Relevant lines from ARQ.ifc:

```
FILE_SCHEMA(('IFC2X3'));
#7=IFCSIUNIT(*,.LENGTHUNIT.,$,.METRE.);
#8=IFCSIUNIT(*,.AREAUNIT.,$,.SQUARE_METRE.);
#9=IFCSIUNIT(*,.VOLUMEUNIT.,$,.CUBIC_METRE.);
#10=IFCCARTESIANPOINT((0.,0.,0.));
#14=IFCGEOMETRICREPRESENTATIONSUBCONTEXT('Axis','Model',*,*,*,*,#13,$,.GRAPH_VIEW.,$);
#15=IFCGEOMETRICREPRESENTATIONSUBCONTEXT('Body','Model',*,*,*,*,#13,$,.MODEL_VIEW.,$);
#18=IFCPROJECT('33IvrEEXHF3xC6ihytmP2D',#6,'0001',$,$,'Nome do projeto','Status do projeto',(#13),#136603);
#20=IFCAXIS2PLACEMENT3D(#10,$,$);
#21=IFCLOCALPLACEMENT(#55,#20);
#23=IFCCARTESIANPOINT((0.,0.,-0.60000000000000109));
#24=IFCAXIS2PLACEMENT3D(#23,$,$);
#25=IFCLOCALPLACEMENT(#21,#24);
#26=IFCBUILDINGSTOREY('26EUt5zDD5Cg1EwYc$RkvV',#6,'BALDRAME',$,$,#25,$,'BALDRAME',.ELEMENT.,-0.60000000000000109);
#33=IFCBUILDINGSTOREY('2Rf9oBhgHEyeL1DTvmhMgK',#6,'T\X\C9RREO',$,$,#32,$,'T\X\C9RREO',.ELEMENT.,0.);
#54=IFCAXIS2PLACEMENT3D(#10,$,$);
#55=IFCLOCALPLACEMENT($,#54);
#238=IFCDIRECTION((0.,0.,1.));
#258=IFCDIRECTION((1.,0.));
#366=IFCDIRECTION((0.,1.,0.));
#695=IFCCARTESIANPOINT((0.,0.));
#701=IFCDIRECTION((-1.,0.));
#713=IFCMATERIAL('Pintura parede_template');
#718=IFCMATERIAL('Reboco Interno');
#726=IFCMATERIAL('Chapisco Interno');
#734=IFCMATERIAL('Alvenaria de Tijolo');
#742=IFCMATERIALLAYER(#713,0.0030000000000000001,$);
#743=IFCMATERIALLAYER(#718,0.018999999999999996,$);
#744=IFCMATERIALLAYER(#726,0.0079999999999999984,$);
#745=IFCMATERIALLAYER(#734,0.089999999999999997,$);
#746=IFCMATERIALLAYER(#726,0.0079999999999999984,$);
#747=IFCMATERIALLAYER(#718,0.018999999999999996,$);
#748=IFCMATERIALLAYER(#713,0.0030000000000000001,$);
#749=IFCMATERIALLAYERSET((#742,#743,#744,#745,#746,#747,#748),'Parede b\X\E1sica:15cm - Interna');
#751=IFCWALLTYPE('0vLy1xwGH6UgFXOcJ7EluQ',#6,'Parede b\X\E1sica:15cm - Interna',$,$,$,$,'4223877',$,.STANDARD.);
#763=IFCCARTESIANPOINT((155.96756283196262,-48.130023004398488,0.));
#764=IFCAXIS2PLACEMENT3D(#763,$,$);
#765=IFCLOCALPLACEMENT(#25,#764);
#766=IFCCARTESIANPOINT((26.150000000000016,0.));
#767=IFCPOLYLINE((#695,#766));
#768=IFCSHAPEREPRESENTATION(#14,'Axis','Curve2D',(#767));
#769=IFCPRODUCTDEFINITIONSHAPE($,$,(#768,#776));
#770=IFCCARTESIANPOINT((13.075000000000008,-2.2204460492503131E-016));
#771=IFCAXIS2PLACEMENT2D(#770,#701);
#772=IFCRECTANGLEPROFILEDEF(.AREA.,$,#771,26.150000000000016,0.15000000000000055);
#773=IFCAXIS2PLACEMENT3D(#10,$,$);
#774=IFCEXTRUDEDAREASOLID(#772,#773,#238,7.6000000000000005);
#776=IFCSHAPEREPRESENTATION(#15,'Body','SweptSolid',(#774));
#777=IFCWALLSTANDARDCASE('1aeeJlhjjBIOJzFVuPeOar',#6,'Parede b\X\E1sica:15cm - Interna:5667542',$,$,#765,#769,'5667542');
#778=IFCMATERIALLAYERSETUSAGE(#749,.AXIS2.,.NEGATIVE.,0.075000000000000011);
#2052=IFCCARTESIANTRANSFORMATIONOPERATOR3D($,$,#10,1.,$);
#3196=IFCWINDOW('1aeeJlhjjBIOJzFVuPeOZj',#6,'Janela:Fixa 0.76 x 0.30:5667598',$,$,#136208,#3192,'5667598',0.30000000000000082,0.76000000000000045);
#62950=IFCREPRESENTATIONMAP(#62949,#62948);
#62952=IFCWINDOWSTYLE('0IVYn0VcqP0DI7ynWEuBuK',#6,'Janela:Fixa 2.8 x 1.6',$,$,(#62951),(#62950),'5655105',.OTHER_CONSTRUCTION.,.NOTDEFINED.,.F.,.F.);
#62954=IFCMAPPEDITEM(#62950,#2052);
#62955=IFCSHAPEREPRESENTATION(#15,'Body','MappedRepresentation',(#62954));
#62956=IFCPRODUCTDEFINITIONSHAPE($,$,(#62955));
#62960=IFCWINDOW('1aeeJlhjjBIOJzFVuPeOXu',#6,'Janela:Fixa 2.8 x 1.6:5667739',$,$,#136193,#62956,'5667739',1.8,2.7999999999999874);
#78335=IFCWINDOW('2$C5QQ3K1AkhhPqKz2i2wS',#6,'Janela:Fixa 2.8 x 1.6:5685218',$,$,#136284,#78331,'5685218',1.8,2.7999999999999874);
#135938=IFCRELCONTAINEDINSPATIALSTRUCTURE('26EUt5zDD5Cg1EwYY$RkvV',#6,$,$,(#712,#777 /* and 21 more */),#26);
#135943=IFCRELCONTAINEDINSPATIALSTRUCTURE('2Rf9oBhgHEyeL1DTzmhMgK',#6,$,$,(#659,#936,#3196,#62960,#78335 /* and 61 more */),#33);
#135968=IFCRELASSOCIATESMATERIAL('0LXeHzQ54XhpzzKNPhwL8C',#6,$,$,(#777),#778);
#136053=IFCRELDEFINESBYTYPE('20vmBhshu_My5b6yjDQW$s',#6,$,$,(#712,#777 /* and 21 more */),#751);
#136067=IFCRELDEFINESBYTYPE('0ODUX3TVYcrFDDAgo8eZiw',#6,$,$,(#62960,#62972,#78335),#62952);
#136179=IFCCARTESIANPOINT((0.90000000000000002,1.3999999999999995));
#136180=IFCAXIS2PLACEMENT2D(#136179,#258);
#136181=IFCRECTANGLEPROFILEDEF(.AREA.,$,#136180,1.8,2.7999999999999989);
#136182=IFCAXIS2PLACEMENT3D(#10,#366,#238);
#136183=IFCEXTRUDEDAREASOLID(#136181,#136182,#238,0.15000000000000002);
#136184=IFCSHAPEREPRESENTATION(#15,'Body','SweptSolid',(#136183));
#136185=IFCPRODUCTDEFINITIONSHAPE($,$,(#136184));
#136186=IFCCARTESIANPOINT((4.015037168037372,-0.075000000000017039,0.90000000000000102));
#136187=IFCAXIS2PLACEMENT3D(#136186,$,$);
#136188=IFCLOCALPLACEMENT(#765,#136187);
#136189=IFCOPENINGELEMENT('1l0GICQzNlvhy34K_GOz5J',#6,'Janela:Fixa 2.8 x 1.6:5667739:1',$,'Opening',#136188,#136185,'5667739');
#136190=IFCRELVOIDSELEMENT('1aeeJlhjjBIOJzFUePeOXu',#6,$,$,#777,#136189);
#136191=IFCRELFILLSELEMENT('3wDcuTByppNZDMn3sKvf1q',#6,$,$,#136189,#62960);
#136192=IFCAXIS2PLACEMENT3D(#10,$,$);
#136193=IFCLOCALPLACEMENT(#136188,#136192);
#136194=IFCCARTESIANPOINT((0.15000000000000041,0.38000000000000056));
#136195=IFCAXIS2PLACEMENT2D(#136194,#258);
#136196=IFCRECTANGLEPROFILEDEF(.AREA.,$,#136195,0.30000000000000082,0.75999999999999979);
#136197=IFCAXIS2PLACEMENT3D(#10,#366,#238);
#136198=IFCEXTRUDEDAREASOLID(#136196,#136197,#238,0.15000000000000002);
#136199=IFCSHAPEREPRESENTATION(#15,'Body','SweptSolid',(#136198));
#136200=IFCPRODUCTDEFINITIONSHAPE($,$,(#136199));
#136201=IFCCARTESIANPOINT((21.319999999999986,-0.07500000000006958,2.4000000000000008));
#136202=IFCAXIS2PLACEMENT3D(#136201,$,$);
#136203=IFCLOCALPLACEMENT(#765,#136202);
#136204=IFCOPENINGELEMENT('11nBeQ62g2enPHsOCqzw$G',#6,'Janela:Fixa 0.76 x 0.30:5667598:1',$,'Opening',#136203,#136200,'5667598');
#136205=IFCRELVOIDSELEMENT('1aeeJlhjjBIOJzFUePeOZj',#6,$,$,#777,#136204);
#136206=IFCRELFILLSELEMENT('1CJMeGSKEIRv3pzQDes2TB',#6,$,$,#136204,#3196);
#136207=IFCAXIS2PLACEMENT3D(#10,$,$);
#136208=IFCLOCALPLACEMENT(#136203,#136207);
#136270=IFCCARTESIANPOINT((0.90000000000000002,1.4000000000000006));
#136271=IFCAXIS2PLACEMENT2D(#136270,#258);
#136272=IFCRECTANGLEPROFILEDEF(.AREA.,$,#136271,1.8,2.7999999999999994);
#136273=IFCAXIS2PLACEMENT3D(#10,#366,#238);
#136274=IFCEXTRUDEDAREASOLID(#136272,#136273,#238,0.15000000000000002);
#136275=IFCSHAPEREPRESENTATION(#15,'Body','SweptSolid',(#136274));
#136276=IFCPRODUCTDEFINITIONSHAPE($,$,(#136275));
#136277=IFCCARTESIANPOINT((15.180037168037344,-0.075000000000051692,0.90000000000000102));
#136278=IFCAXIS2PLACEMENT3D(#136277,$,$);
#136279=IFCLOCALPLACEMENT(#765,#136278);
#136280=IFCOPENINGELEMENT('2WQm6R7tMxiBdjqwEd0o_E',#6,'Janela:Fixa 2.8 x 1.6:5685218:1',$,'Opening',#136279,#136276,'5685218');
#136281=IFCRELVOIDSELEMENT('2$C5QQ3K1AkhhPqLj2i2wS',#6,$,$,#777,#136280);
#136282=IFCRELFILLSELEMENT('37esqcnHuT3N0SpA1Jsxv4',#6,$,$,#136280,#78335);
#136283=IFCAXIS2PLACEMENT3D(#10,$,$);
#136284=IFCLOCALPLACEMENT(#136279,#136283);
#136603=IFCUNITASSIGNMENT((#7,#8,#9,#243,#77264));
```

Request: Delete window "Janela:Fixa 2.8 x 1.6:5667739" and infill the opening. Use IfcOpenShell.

```python
import ifcopenshell
import ifcopenshell.api.feature
import ifcopenshell.api.root
import ifcopenshell.geom
import ifcopenshell.util.shape

model = ifcopenshell.open("ARQ.ifc")
settings = ifcopenshell.geom.settings()


def volume(element):
    """Net volume in cubic metres, openings subtracted."""
    shape = ifcopenshell.geom.create_shape(settings, element)
    return ifcopenshell.util.shape.get_volume(shape.geometry)


window = model.by_guid("1aeeJlhjjBIOJzFVuPeOXu")
opening = window.FillsVoids[0].RelatingOpeningElement
wall = opening.VoidsElements[0].RelatingBuildingElement
before = volume(wall)

ifcopenshell.api.root.remove_product(model, product=window)
ifcopenshell.api.feature.remove_feature(model, feature=opening)

after = volume(wall)

print(f"wall volume {before:.3f} -> {after:.3f} m3")

model.write("ARQ_v2.ifc")
```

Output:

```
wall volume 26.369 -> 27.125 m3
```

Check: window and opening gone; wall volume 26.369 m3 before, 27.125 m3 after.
